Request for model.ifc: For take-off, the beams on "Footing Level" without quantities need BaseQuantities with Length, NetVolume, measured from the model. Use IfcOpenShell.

First a look at what the model holds.

```python
import ifcopenshell
import ifcopenshell.util.element
import ifcopenshell.util.unit

model = ifcopenshell.open("model.ifc")
print(model.schema)
for unit_type in ("LENGTHUNIT", "AREAUNIT", "VOLUMEUNIT"):
    print(unit_type, ifcopenshell.util.unit.calculate_unit_scale(model, unit_type))
storey = next(s for s in model.by_type("IfcBuildingStorey") if s.Name == "Footing Level")
beams = [e for e in ifcopenshell.util.element.get_decomposition(storey) if e.is_a("IfcBeam")]
for e in sorted(beams, key=lambda e: e.id()):
    print(e.id(), e.is_a(), e.Name, list(ifcopenshell.util.element.get_psets(e, qtos_only=True)), sep=" | ")
```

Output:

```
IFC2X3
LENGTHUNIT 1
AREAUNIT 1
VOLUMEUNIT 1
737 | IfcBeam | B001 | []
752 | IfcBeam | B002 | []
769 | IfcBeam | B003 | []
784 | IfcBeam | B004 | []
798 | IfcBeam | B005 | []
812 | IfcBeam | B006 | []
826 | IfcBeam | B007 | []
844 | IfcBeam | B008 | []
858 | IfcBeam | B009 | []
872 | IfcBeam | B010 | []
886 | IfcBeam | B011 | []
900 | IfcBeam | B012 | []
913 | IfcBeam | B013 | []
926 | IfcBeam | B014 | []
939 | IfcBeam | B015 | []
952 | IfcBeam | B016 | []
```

```python
import ifcopenshell
import ifcopenshell.api.pset
import ifcopenshell.geom
import ifcopenshell.util.element
import ifcopenshell.util.shape
import ifcopenshell.util.unit

model = ifcopenshell.open("model.ifc")
unit_scale = ifcopenshell.util.unit.calculate_unit_scale(model)
volume_scale = ifcopenshell.util.unit.calculate_unit_scale(model, "VOLUMEUNIT")
settings = ifcopenshell.geom.settings()

storey = next(s for s in model.by_type("IfcBuildingStorey") if s.Name == "Footing Level")
beams = [e for e in ifcopenshell.util.element.get_decomposition(storey) if e.is_a("IfcBeam")]

for e in sorted(beams, key=lambda e: e.id()):
    if ifcopenshell.util.element.get_psets(e, qtos_only=True, should_inherit=False):
        continue
    # Geometry comes back in metres, in the element's own axes.
    shape = ifcopenshell.geom.create_shape(settings, e)
    values = {
        "Length": ifcopenshell.util.shape.get_max_xyz(shape.geometry) / unit_scale,
        "NetVolume": ifcopenshell.util.shape.get_volume(shape.geometry) / volume_scale,
    }
    qto = ifcopenshell.api.pset.add_qto(model, product=e, name="BaseQuantities")
    ifcopenshell.api.pset.edit_qto(model, qto=qto, properties=values)
    print(e.id(), {k: round(v, 3) for k, v in values.items()})

model.write("model-out.ifc")
```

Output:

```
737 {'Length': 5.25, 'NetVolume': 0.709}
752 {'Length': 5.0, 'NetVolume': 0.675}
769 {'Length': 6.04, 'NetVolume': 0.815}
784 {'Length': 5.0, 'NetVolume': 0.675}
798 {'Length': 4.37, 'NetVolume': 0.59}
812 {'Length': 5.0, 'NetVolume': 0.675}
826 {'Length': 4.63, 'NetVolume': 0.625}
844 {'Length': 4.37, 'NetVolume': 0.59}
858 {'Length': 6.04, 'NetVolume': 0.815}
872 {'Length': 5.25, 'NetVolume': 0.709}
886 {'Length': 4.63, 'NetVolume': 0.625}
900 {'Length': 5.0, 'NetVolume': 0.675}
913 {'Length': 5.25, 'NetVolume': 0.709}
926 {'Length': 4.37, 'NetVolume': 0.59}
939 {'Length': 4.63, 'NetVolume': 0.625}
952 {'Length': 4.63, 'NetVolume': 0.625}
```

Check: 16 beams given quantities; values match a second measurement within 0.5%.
